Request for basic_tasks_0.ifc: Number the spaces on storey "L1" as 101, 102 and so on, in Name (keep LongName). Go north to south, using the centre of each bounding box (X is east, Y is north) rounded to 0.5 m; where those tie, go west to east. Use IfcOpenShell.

First a look at what the model holds.

```python
import ifcopenshell
import ifcopenshell.util.element
import ifcopenshell.util.placement

model = ifcopenshell.open("basic_tasks_0.ifc")
print(model.schema)
storey = next(s for s in model.by_type("IfcBuildingStorey") if s.Name == "L1")
spaces = [e for e in ifcopenshell.util.element.get_decomposition(storey) if e.is_a("IfcSpace")]
for e in sorted(spaces, key=lambda e: e.id()):
    origin = ifcopenshell.util.placement.get_local_placement(e.ObjectPlacement)[:3, 3]
    print(e.id(), e.Name, e.LongName, origin.round(2) + 0.0, sep=" | ")
```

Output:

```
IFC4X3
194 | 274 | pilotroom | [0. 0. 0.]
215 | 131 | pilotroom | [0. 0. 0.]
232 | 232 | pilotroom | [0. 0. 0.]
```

```python
import ifcopenshell
import ifcopenshell.geom
import ifcopenshell.util.element
import ifcopenshell.util.shape

model = ifcopenshell.open("basic_tasks_0.ifc")
settings = ifcopenshell.geom.settings()
settings.set("use-world-coords", True)


def centre(element):
    shape = ifcopenshell.geom.create_shape(settings, element)
    return ifcopenshell.util.shape.get_bbox_centroid(shape.geometry)


storey = next(s for s in model.by_type("IfcBuildingStorey") if s.Name == "L1")
spaces = [e for e in ifcopenshell.util.element.get_decomposition(storey) if e.is_a("IfcSpace")]

# Insertion points can sit at a corner or the storey origin, so sort by the geometry (in metres).
centres = {e: centre(e) for e in spaces}
spaces.sort(key=lambda e: (-round(centres[e][1] / 0.5), centres[e][0]))

for i, e in enumerate(spaces, start=1):
    number = f"1{i:02d}"
    e.Name = number
    print(e.id(), number)

model.write("basic_tasks_0_edited.ifc")
```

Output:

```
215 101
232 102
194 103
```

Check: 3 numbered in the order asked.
